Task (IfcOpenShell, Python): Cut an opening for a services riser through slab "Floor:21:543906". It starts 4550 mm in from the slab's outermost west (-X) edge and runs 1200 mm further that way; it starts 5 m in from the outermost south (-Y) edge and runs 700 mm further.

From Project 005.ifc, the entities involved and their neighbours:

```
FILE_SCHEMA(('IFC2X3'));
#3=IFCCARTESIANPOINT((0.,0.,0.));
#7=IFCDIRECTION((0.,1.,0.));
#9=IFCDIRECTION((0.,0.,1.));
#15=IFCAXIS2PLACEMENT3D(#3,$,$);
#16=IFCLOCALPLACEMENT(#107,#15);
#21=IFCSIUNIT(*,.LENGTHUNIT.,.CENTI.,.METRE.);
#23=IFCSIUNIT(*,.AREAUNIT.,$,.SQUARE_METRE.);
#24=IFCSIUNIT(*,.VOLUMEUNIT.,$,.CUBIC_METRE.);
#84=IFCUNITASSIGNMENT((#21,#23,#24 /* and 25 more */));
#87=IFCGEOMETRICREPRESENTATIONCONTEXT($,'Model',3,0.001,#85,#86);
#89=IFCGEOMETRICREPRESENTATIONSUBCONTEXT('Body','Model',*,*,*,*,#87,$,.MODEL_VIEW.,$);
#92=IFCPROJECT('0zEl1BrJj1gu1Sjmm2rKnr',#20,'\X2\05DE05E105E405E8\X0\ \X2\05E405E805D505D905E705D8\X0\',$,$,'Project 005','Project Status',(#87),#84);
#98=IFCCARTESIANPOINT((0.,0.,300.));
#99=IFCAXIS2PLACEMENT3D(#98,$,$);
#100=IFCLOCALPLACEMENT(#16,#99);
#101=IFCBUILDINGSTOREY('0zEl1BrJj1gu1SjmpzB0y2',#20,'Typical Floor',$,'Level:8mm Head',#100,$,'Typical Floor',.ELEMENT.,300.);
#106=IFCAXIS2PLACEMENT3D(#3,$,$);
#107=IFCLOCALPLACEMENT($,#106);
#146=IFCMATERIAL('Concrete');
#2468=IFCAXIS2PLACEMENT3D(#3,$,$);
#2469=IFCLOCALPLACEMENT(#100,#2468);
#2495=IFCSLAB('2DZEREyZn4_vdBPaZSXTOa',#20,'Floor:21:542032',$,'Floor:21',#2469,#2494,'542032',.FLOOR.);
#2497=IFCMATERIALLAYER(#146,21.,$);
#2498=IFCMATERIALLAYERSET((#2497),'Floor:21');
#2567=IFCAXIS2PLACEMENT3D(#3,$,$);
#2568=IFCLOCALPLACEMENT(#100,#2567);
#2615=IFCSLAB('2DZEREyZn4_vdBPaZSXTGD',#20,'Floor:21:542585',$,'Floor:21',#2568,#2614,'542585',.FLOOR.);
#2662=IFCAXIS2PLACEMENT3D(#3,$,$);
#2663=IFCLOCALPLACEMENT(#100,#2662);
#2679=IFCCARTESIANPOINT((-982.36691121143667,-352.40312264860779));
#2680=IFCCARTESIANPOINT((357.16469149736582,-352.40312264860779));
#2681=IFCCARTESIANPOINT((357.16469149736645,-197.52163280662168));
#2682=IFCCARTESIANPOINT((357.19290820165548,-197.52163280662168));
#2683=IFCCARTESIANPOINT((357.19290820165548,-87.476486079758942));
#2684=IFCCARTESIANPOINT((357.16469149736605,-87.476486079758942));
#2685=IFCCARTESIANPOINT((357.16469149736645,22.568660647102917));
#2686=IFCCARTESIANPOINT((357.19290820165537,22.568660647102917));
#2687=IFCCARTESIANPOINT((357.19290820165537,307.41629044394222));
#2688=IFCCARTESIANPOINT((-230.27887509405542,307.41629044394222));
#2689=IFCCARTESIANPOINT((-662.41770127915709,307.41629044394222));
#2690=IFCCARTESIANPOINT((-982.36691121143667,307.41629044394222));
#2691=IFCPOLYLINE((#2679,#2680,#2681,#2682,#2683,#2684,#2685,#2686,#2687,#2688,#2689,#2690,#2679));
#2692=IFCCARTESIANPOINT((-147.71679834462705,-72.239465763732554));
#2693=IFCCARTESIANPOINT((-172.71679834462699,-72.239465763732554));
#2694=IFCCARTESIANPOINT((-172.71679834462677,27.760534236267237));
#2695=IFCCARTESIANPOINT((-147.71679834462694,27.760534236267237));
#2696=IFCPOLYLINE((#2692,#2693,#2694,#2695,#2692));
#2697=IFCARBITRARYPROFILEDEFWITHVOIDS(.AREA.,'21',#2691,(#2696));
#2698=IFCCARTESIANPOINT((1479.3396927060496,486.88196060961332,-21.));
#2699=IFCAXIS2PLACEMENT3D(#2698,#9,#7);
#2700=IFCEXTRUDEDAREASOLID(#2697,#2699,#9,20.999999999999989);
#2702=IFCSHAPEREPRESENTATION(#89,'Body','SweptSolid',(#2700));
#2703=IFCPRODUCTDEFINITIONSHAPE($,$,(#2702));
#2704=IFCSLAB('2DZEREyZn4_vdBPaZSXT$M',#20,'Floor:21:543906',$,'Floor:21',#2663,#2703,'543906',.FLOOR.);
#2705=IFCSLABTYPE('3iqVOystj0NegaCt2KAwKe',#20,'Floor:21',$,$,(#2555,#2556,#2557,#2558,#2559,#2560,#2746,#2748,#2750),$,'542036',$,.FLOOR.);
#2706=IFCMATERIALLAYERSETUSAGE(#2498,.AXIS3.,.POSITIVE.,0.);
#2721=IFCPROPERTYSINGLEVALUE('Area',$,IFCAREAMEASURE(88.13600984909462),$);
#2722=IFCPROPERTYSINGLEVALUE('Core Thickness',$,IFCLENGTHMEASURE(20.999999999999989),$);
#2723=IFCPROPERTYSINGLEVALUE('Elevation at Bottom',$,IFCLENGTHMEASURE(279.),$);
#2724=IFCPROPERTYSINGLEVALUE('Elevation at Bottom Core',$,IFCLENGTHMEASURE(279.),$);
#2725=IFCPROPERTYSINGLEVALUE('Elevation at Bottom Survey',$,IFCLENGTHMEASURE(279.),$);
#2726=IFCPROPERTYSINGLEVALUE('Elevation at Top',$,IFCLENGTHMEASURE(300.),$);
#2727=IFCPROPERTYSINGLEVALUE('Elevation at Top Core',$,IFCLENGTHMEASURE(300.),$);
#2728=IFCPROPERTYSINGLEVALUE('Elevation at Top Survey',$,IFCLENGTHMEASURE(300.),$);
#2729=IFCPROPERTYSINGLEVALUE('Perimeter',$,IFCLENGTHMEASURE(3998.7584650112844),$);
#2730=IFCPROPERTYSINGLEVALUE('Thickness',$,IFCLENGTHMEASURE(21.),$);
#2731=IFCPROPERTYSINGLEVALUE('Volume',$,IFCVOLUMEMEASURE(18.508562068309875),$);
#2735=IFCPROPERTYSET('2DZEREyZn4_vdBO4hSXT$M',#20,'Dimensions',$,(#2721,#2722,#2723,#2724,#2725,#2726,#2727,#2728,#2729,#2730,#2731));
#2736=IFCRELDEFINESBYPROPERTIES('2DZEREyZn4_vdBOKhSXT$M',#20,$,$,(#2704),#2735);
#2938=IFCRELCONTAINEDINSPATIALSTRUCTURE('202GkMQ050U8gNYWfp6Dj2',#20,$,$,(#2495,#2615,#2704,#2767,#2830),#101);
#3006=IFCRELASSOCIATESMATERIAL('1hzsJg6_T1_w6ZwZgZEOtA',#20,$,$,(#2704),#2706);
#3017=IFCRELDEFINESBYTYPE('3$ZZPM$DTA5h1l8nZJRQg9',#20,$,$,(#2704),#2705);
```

```python
import numpy as np
import ifcopenshell
import ifcopenshell.api.feature
import ifcopenshell.api.geometry
import ifcopenshell.api.pset
import ifcopenshell.api.root
import ifcopenshell.geom
import ifcopenshell.util.element
import ifcopenshell.util.placement
import ifcopenshell.util.representation
import ifcopenshell.util.shape
import ifcopenshell.util.unit

model = ifcopenshell.open("Project 005.ifc")
unit_scale = ifcopenshell.util.unit.calculate_unit_scale(model)
area_scale = ifcopenshell.util.unit.calculate_unit_scale(model, "AREAUNIT")
volume_scale = ifcopenshell.util.unit.calculate_unit_scale(model, "VOLUMEUNIT")
settings = ifcopenshell.geom.settings()


def volume(element):
    """Net volume in cubic metres, openings subtracted."""
    shape = ifcopenshell.geom.create_shape(settings, element)
    return ifcopenshell.util.shape.get_volume(shape.geometry)


slab = model.by_id(2704)
before = volume(slab)

# Extent in the slab's own axes, in metres. The edges named are its -X and -Y sides.
slab_shape = ifcopenshell.geom.create_shape(settings, slab)
vertices = ifcopenshell.util.shape.get_vertices(slab_shape.geometry)
x_min, y_min, bottom = vertices.min(axis=0)
top = vertices[:, 2].max()

opening = ifcopenshell.api.root.create_entity(model, ifc_class="IfcOpeningElement", name="Services riser opening")
context = ifcopenshell.util.representation.get_context(model, "Model", "Body", "MODEL_VIEW")
width, depth = 1.2, 0.7
outline = [(0.0, 0.0), (width, 0.0), (width, depth), (0.0, depth), (0.0, 0.0)]
# Overshoot both faces by 50 mm so the cut is clean.
shape = ifcopenshell.api.geometry.add_slab_representation(
    model, context=context, depth=top - bottom + 0.1, polyline=outline
)
ifcopenshell.api.geometry.assign_representation(model, product=opening, representation=shape)

matrix = ifcopenshell.util.placement.get_local_placement(slab.ObjectPlacement)
matrix[:, 3] = matrix @ np.append(np.array([x_min + 4.55, y_min + 5, bottom - 0.05]) / unit_scale, 1.0)
ifcopenshell.api.geometry.edit_object_placement(model, product=opening, matrix=matrix, is_si=False)
ifcopenshell.api.feature.add_feature(model, feature=opening, element=slab)

after = volume(slab)

# Update the slab's stored quantities.
pset = model.by_id(ifcopenshell.util.element.get_pset(slab, "Dimensions", should_inherit=False)["id"])
ifcopenshell.api.pset.edit_pset(model, pset=pset, properties={
    "Area": model.create_entity("IfcAreaMeasure", after / (top - bottom) / area_scale),
    "Volume": model.create_entity("IfcVolumeMeasure", after / volume_scale),
})

print(f"slab volume {before:.3f} -> {after:.3f} m3")

model.write("Project 005_edited.ifc")
```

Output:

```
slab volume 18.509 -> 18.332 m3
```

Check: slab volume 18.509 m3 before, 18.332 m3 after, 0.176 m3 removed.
